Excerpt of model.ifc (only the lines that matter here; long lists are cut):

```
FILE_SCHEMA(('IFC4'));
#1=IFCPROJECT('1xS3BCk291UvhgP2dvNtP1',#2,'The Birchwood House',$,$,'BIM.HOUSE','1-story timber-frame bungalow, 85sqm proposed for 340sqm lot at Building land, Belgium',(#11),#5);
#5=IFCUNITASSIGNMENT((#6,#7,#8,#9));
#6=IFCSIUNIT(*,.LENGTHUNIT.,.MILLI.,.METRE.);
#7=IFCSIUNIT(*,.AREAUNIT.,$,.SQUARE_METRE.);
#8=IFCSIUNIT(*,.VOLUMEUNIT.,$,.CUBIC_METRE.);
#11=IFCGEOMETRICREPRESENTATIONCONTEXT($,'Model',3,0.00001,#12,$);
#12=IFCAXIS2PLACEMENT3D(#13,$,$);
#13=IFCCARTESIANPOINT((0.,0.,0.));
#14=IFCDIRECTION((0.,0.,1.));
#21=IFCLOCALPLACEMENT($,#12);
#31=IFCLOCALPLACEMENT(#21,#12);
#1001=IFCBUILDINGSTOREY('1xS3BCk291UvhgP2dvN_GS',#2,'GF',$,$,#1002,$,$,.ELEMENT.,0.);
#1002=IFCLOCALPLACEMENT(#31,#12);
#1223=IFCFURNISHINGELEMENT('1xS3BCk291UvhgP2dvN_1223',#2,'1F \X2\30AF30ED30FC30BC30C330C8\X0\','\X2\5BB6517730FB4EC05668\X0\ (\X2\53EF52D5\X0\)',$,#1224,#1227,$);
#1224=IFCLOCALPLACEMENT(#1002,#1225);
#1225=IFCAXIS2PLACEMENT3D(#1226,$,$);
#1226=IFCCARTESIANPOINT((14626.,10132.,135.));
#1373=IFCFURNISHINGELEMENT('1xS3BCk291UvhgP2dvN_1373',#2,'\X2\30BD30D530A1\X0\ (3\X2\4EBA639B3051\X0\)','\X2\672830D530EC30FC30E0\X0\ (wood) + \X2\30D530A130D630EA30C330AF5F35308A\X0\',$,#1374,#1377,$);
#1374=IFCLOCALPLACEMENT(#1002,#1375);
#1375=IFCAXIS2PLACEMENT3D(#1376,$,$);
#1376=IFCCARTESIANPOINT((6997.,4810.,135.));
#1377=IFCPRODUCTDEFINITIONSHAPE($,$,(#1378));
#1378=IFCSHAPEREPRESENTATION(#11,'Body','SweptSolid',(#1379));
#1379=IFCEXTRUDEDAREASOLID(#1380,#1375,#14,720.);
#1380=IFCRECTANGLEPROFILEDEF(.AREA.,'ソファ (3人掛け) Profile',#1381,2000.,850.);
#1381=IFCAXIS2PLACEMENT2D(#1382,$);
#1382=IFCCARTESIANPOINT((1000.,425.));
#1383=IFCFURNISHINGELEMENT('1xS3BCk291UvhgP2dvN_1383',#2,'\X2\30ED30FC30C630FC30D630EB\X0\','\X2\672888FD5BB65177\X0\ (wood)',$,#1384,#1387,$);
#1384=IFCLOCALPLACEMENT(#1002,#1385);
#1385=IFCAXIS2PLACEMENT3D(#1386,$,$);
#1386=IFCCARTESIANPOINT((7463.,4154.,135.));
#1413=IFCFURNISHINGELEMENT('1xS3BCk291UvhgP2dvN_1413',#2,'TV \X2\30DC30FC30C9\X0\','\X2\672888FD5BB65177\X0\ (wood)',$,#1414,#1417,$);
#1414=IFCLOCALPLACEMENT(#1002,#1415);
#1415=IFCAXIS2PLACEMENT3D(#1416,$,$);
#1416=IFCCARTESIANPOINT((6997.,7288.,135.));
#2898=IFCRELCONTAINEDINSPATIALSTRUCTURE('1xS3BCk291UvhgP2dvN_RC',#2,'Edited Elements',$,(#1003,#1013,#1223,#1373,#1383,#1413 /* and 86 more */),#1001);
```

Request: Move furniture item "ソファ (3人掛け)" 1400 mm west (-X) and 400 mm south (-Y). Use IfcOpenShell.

```python
import ifcopenshell
import ifcopenshell.api.geometry
import ifcopenshell.util.placement
import ifcopenshell.util.unit

model = ifcopenshell.open("model.ifc")
unit_scale = ifcopenshell.util.unit.calculate_unit_scale(model)

item = model.by_id(1373)
matrix = ifcopenshell.util.placement.get_local_placement(item.ObjectPlacement)
matrix[0, 3] -= 1.4 / unit_scale
matrix[1, 3] -= 0.4 / unit_scale
ifcopenshell.api.geometry.edit_object_placement(model, product=item, matrix=matrix, is_si=False)

print(ifcopenshell.util.placement.get_local_placement(item.ObjectPlacement).round(3) + 0.0)

model.write("model_rev.ifc")
```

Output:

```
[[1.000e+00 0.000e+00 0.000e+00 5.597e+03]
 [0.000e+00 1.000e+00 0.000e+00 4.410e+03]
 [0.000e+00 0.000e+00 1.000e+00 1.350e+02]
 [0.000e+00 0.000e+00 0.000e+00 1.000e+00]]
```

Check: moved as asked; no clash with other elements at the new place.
